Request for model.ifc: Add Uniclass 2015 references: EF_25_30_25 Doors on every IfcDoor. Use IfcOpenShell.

First a look at what the model holds.

```python
import ifcopenshell

model = ifcopenshell.open("model.ifc")
print(model.schema)
print("classifications:", [c.Name for c in model.by_type("IfcClassification")])
for ifc_class in ("IfcDoor", "IfcRoof", "IfcStair", "IfcWall", "IfcWindow"):
    print(ifc_class, len(model.by_type(ifc_class)))
```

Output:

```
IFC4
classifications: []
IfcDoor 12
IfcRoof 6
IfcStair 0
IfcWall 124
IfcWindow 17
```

```python
import ifcopenshell
import ifcopenshell.api.classification

model = ifcopenshell.open("model.ifc")

system = ifcopenshell.api.classification.add_classification(model, classification="Uniclass 2015")

codes = {
    "IfcDoor": ("EF_25_30_25", "Doors"),
}
for ifc_class, (code, name) in codes.items():
    products = model.by_type(ifc_class)
    ifcopenshell.api.classification.add_reference(
        model, products=products, classification=system, identification=code, name=name
    )
    print(code, len(products))

model.write("model_edited.ifc")
```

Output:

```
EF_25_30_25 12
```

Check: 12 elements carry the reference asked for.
